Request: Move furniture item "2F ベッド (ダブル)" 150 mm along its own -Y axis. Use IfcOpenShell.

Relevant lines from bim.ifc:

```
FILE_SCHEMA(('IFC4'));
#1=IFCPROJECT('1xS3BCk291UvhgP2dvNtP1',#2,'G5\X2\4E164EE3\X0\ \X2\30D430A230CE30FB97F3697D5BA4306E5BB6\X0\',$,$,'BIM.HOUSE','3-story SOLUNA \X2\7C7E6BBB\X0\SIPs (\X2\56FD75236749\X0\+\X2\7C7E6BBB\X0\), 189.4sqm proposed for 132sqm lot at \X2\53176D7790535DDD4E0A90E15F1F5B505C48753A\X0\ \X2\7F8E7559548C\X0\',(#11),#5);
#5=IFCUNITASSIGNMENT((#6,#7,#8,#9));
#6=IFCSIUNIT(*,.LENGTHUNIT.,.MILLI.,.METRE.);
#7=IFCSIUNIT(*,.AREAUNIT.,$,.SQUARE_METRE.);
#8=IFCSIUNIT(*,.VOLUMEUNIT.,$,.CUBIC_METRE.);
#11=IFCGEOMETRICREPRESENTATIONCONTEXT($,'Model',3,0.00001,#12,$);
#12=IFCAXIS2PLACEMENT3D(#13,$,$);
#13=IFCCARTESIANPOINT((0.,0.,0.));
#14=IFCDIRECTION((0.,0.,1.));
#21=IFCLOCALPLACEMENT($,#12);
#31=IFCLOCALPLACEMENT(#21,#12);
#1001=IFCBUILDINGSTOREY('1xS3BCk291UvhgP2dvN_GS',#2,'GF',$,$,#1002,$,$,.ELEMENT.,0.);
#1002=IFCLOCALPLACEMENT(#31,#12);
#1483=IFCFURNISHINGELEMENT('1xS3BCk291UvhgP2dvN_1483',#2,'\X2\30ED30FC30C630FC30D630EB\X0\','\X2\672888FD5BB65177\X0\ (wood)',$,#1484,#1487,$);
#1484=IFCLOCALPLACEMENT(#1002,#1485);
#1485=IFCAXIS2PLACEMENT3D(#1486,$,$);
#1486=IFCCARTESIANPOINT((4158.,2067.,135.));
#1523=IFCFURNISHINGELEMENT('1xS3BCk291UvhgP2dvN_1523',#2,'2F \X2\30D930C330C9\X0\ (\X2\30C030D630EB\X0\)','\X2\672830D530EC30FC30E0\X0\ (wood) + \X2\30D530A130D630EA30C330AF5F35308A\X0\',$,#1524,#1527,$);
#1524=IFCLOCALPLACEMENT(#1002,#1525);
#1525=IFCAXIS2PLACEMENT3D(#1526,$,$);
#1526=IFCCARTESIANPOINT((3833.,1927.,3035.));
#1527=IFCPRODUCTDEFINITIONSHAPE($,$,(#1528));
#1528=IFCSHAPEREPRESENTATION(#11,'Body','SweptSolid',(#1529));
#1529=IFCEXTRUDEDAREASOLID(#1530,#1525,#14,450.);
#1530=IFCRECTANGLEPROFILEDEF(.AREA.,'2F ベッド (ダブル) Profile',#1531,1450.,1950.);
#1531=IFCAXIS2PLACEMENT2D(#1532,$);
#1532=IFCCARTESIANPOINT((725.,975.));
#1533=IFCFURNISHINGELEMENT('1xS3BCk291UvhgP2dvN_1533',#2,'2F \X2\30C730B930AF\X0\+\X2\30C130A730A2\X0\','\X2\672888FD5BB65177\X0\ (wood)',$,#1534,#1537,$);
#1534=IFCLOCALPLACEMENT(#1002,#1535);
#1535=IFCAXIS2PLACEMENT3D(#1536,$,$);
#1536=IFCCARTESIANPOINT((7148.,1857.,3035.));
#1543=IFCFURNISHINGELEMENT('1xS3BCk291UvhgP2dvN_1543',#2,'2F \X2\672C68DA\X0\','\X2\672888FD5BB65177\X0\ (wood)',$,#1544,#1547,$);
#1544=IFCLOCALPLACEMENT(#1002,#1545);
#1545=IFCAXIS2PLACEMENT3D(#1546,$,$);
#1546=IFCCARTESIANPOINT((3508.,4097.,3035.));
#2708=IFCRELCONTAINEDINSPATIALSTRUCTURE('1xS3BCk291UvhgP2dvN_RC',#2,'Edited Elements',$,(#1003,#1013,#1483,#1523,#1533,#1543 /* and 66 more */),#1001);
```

```python
import ifcopenshell
import ifcopenshell.api.geometry
import ifcopenshell.util.placement
import ifcopenshell.util.unit

model = ifcopenshell.open("bim.ifc")
unit_scale = ifcopenshell.util.unit.calculate_unit_scale(model)

item = model.by_guid("1xS3BCk291UvhgP2dvN_1523")
matrix = ifcopenshell.util.placement.get_local_placement(item.ObjectPlacement)
matrix[:3, 3] -= matrix[:3, 1] * 0.15 / unit_scale
ifcopenshell.api.geometry.edit_object_placement(model, product=item, matrix=matrix, is_si=False)

print(ifcopenshell.util.placement.get_local_placement(item.ObjectPlacement).round(3) + 0.0)

model.write("bim_rev.ifc")
```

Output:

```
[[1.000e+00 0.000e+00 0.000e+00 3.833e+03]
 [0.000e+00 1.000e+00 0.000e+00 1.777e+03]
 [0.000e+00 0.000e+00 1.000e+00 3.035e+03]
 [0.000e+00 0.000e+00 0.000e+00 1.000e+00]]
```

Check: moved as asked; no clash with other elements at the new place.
